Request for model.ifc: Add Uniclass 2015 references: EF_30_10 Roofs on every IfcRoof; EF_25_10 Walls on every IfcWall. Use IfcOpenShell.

First a look at what the model holds.

```python
import ifcopenshell

model = ifcopenshell.open("model.ifc")
print(model.schema)
print("classifications:", [c.Name for c in model.by_type("IfcClassification")])
for ifc_class in ("IfcDoor", "IfcRoof", "IfcStair", "IfcWall", "IfcWindow"):
    print(ifc_class, len(model.by_type(ifc_class)))
```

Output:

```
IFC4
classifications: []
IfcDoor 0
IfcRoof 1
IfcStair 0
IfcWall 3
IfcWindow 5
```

```python
import ifcopenshell
import ifcopenshell.api.classification

model = ifcopenshell.open("model.ifc")

system = ifcopenshell.api.classification.add_classification(model, classification="Uniclass 2015")

codes = {
    "IfcRoof": ("EF_30_10", "Roofs"),
    "IfcWall": ("EF_25_10", "Walls"),
}
for ifc_class, (code, name) in codes.items():
    products = model.by_type(ifc_class)
    ifcopenshell.api.classification.add_reference(
        model, products=products, classification=system, identification=code, name=name
    )
    print(code, len(products))

model.write("model_v2.ifc")
```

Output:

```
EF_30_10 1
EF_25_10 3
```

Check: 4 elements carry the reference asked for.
